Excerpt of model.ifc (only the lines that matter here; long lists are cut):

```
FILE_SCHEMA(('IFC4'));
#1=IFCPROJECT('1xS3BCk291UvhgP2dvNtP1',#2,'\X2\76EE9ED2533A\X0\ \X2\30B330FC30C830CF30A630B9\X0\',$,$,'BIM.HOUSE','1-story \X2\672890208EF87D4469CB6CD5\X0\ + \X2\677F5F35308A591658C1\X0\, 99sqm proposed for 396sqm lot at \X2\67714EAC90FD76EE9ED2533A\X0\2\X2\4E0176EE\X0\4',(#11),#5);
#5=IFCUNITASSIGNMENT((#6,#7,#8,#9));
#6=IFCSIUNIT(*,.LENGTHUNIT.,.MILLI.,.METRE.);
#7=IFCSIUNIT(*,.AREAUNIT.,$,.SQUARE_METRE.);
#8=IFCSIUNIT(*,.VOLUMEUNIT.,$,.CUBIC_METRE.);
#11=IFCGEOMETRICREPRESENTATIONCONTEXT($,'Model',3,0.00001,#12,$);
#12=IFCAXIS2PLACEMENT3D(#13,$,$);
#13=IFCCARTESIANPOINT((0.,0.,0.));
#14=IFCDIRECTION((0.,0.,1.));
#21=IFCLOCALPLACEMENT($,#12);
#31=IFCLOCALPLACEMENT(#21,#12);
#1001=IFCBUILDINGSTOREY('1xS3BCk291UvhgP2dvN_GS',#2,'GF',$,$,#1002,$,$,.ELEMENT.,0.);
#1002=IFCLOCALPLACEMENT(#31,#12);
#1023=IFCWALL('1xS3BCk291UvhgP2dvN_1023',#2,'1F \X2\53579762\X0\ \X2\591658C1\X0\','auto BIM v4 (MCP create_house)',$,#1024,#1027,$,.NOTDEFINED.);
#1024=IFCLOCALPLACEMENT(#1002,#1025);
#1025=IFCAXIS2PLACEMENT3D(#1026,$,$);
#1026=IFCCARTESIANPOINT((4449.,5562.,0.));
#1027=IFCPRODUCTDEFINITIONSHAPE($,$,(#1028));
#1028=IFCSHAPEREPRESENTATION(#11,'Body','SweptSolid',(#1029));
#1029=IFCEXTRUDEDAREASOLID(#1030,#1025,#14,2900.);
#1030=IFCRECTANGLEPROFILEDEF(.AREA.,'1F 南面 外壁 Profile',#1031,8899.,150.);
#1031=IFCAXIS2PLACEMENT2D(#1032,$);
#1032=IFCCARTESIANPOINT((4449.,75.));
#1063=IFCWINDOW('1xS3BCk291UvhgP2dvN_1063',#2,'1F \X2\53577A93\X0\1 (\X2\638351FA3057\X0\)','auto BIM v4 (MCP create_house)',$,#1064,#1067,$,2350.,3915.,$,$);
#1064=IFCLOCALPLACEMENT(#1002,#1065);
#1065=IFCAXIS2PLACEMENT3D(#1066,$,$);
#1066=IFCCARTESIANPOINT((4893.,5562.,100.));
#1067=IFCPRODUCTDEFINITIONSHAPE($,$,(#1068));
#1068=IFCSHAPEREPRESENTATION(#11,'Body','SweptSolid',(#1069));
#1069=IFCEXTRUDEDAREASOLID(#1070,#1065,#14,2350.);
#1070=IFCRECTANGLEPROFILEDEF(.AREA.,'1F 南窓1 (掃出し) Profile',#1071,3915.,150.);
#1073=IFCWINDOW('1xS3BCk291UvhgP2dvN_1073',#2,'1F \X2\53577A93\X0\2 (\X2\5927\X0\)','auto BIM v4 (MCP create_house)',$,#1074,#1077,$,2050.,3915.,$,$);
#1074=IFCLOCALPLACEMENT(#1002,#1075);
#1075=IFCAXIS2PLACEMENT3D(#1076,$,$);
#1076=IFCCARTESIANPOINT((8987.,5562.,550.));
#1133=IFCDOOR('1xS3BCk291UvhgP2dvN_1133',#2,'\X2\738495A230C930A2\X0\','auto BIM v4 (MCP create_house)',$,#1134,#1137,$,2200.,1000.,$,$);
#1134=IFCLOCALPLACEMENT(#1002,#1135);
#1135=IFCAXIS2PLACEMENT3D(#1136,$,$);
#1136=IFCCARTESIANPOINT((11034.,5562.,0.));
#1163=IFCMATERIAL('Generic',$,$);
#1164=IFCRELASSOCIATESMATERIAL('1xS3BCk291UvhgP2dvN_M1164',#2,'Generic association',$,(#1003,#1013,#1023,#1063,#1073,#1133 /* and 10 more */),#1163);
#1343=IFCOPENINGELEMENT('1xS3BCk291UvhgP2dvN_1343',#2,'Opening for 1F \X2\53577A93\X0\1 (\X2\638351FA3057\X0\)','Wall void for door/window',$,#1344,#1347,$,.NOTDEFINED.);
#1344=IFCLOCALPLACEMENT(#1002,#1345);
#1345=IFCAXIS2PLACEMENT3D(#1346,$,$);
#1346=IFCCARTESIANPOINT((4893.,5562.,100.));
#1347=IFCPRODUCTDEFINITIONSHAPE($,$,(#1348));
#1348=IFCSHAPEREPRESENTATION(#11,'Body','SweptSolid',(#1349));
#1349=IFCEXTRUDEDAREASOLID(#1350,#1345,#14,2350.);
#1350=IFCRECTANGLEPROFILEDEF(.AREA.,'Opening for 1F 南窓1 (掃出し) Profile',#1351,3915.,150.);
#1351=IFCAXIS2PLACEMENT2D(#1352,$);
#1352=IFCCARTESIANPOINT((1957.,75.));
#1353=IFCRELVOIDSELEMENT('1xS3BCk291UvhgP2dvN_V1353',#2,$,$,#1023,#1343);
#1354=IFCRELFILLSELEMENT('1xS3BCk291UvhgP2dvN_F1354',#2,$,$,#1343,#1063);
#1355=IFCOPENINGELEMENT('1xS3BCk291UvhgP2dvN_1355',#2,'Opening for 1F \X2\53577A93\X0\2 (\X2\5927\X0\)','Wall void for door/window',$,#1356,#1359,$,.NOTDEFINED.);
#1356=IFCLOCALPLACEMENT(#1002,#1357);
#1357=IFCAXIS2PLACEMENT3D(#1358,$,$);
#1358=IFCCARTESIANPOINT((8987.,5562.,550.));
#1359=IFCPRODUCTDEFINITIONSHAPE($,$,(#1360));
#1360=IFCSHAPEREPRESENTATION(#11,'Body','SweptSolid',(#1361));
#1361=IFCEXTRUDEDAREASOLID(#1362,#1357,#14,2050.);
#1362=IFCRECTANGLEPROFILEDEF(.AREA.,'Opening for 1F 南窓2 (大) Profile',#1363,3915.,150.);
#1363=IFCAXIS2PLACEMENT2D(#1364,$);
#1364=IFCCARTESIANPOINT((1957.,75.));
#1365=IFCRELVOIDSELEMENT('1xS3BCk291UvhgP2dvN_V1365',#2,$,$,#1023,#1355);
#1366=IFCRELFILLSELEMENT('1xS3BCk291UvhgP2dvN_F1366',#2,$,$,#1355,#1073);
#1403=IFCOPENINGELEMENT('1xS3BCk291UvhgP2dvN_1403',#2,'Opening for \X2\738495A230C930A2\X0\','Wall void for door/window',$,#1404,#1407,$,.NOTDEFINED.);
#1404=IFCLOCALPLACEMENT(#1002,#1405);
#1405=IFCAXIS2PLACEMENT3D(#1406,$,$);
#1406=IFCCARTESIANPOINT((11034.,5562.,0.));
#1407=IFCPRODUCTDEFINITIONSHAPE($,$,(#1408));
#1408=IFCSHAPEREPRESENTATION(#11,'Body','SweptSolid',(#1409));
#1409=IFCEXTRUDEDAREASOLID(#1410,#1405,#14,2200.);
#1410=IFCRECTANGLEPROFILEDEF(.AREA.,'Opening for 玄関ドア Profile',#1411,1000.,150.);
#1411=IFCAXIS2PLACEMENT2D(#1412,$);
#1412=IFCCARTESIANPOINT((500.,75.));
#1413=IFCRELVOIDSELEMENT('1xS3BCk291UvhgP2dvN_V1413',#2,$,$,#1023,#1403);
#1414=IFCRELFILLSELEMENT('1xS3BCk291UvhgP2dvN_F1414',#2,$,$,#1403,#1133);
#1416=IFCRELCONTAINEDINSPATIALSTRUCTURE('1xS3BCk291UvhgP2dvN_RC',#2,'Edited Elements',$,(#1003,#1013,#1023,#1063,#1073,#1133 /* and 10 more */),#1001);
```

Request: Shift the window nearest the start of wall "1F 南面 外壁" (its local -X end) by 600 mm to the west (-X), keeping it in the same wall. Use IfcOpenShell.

```python
import ifcopenshell
import ifcopenshell.api.geometry
import ifcopenshell.util.placement
import ifcopenshell.util.unit

model = ifcopenshell.open("model.ifc")
unit_scale = ifcopenshell.util.unit.calculate_unit_scale(model)

window = model.by_id(1063)
opening = window.FillsVoids[0].RelatingOpeningElement
wall = opening.VoidsElements[0].RelatingBuildingElement

wall_matrix = ifcopenshell.util.placement.get_local_placement(wall.ObjectPlacement)
shift = wall_matrix[:3, 0] * -0.6 / unit_scale
before = ifcopenshell.util.placement.get_local_placement(window.ObjectPlacement)[:3, 3].copy()

# The window is not placed relative to its opening, so move both.
for product in (opening, window):
    matrix = ifcopenshell.util.placement.get_local_placement(product.ObjectPlacement)
    matrix[:3, 3] += shift
    ifcopenshell.api.geometry.edit_object_placement(model, product=product, matrix=matrix, is_si=False)

after = ifcopenshell.util.placement.get_local_placement(window.ObjectPlacement)[:3, 3]
print("window moved by", (after - before).round(3) + 0.0)

model.write("model_v2.ifc")
```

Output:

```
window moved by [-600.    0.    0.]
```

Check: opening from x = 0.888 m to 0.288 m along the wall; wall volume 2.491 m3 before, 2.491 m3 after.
